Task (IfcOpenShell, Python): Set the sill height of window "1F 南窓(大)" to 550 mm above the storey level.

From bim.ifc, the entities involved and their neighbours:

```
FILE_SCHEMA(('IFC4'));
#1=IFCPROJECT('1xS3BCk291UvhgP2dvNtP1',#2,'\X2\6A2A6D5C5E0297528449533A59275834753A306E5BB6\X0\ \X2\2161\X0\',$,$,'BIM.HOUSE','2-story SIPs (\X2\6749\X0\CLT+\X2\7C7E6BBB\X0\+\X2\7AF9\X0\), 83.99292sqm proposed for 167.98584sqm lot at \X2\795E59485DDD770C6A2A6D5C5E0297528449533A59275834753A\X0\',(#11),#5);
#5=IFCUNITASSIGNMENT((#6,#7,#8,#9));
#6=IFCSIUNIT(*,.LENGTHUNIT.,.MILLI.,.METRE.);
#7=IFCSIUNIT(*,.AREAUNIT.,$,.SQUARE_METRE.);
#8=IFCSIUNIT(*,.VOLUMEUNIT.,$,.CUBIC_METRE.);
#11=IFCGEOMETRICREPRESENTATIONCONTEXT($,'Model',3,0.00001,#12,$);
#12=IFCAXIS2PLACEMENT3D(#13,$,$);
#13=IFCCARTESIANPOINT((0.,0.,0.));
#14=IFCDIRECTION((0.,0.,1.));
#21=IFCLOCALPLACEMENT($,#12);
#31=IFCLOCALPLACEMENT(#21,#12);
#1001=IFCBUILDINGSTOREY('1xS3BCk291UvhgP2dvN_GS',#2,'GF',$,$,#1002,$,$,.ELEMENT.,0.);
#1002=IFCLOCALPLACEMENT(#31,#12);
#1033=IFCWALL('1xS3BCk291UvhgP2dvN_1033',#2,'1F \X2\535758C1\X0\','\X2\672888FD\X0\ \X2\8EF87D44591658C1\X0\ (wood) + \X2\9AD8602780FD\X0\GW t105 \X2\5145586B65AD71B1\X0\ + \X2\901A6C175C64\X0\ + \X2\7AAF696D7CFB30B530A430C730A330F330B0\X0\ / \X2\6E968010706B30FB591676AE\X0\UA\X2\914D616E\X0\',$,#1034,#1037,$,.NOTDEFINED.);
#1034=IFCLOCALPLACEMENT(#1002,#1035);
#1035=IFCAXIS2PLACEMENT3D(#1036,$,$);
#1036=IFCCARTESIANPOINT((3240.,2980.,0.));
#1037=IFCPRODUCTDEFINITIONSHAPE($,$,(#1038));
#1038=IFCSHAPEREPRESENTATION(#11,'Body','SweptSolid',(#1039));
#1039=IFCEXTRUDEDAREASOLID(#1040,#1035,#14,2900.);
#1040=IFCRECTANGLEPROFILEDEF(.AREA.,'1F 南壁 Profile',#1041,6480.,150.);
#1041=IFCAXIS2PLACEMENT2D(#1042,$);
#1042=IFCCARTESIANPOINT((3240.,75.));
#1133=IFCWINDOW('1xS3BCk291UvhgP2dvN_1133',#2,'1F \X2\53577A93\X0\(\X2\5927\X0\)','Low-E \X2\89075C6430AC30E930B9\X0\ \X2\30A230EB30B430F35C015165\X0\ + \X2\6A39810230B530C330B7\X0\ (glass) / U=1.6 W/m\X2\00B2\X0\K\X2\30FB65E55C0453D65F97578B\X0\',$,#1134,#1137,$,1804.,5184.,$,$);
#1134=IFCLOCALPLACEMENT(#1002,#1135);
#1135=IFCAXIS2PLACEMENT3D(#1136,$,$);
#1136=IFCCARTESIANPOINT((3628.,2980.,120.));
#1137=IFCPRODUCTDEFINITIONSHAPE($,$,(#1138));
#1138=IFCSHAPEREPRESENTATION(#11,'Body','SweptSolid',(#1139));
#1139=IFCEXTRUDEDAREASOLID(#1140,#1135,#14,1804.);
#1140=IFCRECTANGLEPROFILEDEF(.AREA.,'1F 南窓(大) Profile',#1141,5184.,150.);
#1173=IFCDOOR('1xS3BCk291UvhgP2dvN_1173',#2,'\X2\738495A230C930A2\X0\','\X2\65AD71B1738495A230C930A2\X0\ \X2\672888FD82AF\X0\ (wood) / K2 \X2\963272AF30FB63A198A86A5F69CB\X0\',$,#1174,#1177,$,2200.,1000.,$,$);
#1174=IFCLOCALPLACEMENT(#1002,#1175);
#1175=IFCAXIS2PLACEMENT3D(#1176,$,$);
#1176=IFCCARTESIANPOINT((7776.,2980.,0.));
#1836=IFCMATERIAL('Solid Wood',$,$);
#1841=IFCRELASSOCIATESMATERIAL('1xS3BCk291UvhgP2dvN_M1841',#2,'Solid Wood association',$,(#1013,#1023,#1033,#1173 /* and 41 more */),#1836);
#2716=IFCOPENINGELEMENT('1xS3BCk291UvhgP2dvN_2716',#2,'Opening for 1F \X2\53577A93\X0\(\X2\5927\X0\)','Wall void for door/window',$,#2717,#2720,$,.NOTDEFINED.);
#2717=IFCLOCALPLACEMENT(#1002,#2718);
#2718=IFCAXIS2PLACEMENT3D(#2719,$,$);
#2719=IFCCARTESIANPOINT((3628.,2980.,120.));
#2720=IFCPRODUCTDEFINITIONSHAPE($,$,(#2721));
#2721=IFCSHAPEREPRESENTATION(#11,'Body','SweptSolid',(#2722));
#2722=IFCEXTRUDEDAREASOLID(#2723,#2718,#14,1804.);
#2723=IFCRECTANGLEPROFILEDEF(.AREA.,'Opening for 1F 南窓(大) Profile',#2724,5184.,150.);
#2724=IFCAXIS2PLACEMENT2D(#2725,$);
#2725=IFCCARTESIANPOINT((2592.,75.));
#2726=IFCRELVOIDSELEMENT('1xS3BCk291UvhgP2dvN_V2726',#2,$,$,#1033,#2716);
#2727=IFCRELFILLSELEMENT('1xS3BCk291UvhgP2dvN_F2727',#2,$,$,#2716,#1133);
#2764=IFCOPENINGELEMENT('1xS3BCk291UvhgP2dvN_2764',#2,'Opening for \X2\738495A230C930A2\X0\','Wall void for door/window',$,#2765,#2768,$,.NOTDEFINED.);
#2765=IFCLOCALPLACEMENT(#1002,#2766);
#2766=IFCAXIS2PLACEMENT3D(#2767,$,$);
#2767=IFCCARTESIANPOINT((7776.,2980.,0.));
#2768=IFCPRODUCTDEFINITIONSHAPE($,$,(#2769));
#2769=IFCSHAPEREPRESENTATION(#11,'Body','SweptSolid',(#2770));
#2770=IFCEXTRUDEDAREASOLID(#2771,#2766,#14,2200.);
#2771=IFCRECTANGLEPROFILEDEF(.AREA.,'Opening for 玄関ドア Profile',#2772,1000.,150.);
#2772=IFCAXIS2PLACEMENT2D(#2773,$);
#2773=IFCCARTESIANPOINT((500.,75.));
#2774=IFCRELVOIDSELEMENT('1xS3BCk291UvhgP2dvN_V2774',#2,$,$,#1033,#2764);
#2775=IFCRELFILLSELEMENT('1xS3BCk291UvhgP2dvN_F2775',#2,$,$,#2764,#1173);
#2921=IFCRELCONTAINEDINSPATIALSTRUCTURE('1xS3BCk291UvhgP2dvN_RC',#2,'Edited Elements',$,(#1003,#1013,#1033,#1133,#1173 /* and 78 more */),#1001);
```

```python
import numpy as np
import ifcopenshell
import ifcopenshell.api.geometry
import ifcopenshell.geom
import ifcopenshell.util.element
import ifcopenshell.util.placement
import ifcopenshell.util.shape
import ifcopenshell.util.unit

model = ifcopenshell.open("bim.ifc")
unit_scale = ifcopenshell.util.unit.calculate_unit_scale(model)

window = model.by_id(1133)
opening = window.FillsVoids[0].RelatingOpeningElement
storey = ifcopenshell.util.element.get_container(window, ifc_class="IfcBuildingStorey")
level = ifcopenshell.util.placement.get_local_placement(storey.ObjectPlacement)[2, 3]

# The opening's origin need not be at the sill, so measure its lowest point.
shape = ifcopenshell.geom.create_shape(ifcopenshell.geom.settings(), opening)
bottom = ifcopenshell.util.shape.get_shape_bottom_elevation(shape, shape.geometry) / unit_scale
dz = level + 0.55 / unit_scale - bottom

shift = np.array([0.0, 0.0, dz])
# The window is not placed relative to its opening, so move both.
for product in (opening, window):
    matrix = ifcopenshell.util.placement.get_local_placement(product.ObjectPlacement)
    matrix[:3, 3] += shift
    ifcopenshell.api.geometry.edit_object_placement(model, product=product, matrix=matrix, is_si=False)

print(f"moved by {dz * unit_scale:+.3f} m")

model.write("bim-out.ifc")
```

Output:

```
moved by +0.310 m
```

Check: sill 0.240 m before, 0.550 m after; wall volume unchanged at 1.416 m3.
